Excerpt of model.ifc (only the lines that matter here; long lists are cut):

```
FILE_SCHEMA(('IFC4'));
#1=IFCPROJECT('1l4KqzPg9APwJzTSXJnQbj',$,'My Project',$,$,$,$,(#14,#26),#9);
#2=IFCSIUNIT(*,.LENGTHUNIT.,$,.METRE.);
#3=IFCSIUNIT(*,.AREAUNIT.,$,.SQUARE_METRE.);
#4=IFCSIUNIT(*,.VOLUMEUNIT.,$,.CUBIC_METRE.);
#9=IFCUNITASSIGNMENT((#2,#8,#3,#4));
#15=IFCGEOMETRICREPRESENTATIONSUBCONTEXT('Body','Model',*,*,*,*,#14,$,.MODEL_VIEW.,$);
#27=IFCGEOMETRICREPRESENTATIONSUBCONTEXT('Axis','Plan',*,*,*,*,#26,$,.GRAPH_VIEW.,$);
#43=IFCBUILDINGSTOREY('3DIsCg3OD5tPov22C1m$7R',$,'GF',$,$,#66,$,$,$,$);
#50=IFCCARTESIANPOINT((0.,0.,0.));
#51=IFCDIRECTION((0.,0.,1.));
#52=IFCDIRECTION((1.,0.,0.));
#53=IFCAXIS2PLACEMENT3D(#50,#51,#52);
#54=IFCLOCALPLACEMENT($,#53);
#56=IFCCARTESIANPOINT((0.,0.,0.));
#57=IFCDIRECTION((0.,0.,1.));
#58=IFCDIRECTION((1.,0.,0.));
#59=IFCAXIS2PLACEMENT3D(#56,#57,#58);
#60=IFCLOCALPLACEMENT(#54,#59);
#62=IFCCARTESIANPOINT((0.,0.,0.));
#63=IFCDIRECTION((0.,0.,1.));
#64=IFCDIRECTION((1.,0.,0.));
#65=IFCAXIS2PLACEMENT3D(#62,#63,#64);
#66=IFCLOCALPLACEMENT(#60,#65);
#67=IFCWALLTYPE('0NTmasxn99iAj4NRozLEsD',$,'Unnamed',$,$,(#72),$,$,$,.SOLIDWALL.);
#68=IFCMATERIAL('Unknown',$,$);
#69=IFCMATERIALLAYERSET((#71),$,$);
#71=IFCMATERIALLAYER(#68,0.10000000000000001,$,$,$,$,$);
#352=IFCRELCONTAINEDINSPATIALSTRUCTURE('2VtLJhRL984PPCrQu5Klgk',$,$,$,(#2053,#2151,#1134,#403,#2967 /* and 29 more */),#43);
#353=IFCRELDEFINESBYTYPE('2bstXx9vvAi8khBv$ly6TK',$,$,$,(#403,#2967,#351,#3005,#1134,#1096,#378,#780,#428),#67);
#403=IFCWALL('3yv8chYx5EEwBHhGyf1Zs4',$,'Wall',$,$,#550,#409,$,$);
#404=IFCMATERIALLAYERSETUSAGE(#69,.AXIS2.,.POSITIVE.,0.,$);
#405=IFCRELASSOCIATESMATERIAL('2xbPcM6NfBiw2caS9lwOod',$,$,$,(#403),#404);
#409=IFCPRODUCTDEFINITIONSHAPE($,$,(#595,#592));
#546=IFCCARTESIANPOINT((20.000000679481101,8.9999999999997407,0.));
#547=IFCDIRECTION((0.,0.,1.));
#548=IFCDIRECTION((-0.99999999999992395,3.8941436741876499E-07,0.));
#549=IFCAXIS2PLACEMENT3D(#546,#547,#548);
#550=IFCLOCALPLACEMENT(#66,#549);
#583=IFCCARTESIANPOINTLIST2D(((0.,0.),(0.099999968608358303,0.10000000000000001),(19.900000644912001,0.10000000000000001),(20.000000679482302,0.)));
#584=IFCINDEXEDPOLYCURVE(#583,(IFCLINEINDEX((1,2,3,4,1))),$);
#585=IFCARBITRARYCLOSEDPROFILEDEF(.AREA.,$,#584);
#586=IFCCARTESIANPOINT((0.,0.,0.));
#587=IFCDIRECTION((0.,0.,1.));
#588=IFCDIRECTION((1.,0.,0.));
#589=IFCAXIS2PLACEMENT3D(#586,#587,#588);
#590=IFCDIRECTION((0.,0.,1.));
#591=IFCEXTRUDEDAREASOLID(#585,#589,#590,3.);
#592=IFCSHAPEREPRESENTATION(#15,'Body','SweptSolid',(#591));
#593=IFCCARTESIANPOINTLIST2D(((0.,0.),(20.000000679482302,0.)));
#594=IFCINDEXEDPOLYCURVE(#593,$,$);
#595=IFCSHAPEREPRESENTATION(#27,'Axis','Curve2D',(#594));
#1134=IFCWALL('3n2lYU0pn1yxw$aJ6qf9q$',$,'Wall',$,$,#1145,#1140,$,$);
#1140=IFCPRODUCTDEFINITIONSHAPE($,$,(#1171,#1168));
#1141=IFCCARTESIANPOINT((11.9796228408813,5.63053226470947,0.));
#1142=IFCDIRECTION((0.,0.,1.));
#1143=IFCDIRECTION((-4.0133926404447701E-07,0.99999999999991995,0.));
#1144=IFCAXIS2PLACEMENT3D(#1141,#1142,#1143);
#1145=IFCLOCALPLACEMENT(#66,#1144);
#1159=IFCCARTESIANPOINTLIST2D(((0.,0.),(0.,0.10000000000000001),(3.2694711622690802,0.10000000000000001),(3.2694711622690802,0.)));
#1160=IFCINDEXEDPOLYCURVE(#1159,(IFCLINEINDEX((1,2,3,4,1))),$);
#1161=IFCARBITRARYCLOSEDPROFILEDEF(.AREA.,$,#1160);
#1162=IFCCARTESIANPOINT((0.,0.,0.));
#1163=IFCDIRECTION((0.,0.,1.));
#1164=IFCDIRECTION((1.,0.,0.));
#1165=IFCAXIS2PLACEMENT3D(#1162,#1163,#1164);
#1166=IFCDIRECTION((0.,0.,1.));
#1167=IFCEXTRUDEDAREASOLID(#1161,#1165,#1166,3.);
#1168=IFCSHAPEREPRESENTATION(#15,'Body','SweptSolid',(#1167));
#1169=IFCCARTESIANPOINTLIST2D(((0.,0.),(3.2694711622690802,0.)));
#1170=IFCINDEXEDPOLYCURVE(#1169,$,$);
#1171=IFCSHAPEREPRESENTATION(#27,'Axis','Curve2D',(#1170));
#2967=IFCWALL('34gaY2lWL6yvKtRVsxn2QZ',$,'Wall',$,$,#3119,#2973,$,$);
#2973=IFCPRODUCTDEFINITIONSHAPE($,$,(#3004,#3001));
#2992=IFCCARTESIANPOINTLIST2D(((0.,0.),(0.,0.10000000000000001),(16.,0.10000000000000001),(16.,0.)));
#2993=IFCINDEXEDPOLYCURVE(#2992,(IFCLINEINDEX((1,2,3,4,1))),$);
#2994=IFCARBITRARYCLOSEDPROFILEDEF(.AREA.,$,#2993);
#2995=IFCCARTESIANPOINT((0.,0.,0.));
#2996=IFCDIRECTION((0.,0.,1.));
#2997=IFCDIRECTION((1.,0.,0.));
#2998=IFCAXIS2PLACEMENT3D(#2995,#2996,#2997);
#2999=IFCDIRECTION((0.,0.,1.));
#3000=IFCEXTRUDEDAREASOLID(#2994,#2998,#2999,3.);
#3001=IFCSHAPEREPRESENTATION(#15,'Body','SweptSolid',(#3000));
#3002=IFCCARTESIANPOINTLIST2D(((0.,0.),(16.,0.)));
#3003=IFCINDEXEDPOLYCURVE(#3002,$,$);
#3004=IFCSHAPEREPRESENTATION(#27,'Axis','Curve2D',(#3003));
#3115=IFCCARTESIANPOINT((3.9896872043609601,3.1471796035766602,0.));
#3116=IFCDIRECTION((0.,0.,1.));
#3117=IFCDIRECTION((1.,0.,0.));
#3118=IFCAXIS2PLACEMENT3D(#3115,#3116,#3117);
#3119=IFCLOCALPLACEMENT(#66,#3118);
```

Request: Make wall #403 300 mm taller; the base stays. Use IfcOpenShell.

```python
import ifcopenshell
import ifcopenshell.geom
import ifcopenshell.util.representation
import ifcopenshell.util.shape
import ifcopenshell.util.unit

model = ifcopenshell.open("model.ifc")
unit_scale = ifcopenshell.util.unit.calculate_unit_scale(model)
settings = ifcopenshell.geom.settings()


def volume(element):
    """Net volume in cubic metres, openings subtracted."""
    shape = ifcopenshell.geom.create_shape(settings, element)
    return ifcopenshell.util.shape.get_volume(shape.geometry)


wall = model.by_guid("3yv8chYx5EEwBHhGyf1Zs4")
before = volume(wall)

body = ifcopenshell.util.representation.get_representation(wall, "Model", "Body")
solid = body.Items[0]
old_height = solid.Depth
solid.Depth += 0.3 / unit_scale
after = volume(wall)

print(f"height {old_height:g} -> {solid.Depth:g}, volume {before:.3f} -> {after:.3f} m3")

model.write("model_v2.ifc")
```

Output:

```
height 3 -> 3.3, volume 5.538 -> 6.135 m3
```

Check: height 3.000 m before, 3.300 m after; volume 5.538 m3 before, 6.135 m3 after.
